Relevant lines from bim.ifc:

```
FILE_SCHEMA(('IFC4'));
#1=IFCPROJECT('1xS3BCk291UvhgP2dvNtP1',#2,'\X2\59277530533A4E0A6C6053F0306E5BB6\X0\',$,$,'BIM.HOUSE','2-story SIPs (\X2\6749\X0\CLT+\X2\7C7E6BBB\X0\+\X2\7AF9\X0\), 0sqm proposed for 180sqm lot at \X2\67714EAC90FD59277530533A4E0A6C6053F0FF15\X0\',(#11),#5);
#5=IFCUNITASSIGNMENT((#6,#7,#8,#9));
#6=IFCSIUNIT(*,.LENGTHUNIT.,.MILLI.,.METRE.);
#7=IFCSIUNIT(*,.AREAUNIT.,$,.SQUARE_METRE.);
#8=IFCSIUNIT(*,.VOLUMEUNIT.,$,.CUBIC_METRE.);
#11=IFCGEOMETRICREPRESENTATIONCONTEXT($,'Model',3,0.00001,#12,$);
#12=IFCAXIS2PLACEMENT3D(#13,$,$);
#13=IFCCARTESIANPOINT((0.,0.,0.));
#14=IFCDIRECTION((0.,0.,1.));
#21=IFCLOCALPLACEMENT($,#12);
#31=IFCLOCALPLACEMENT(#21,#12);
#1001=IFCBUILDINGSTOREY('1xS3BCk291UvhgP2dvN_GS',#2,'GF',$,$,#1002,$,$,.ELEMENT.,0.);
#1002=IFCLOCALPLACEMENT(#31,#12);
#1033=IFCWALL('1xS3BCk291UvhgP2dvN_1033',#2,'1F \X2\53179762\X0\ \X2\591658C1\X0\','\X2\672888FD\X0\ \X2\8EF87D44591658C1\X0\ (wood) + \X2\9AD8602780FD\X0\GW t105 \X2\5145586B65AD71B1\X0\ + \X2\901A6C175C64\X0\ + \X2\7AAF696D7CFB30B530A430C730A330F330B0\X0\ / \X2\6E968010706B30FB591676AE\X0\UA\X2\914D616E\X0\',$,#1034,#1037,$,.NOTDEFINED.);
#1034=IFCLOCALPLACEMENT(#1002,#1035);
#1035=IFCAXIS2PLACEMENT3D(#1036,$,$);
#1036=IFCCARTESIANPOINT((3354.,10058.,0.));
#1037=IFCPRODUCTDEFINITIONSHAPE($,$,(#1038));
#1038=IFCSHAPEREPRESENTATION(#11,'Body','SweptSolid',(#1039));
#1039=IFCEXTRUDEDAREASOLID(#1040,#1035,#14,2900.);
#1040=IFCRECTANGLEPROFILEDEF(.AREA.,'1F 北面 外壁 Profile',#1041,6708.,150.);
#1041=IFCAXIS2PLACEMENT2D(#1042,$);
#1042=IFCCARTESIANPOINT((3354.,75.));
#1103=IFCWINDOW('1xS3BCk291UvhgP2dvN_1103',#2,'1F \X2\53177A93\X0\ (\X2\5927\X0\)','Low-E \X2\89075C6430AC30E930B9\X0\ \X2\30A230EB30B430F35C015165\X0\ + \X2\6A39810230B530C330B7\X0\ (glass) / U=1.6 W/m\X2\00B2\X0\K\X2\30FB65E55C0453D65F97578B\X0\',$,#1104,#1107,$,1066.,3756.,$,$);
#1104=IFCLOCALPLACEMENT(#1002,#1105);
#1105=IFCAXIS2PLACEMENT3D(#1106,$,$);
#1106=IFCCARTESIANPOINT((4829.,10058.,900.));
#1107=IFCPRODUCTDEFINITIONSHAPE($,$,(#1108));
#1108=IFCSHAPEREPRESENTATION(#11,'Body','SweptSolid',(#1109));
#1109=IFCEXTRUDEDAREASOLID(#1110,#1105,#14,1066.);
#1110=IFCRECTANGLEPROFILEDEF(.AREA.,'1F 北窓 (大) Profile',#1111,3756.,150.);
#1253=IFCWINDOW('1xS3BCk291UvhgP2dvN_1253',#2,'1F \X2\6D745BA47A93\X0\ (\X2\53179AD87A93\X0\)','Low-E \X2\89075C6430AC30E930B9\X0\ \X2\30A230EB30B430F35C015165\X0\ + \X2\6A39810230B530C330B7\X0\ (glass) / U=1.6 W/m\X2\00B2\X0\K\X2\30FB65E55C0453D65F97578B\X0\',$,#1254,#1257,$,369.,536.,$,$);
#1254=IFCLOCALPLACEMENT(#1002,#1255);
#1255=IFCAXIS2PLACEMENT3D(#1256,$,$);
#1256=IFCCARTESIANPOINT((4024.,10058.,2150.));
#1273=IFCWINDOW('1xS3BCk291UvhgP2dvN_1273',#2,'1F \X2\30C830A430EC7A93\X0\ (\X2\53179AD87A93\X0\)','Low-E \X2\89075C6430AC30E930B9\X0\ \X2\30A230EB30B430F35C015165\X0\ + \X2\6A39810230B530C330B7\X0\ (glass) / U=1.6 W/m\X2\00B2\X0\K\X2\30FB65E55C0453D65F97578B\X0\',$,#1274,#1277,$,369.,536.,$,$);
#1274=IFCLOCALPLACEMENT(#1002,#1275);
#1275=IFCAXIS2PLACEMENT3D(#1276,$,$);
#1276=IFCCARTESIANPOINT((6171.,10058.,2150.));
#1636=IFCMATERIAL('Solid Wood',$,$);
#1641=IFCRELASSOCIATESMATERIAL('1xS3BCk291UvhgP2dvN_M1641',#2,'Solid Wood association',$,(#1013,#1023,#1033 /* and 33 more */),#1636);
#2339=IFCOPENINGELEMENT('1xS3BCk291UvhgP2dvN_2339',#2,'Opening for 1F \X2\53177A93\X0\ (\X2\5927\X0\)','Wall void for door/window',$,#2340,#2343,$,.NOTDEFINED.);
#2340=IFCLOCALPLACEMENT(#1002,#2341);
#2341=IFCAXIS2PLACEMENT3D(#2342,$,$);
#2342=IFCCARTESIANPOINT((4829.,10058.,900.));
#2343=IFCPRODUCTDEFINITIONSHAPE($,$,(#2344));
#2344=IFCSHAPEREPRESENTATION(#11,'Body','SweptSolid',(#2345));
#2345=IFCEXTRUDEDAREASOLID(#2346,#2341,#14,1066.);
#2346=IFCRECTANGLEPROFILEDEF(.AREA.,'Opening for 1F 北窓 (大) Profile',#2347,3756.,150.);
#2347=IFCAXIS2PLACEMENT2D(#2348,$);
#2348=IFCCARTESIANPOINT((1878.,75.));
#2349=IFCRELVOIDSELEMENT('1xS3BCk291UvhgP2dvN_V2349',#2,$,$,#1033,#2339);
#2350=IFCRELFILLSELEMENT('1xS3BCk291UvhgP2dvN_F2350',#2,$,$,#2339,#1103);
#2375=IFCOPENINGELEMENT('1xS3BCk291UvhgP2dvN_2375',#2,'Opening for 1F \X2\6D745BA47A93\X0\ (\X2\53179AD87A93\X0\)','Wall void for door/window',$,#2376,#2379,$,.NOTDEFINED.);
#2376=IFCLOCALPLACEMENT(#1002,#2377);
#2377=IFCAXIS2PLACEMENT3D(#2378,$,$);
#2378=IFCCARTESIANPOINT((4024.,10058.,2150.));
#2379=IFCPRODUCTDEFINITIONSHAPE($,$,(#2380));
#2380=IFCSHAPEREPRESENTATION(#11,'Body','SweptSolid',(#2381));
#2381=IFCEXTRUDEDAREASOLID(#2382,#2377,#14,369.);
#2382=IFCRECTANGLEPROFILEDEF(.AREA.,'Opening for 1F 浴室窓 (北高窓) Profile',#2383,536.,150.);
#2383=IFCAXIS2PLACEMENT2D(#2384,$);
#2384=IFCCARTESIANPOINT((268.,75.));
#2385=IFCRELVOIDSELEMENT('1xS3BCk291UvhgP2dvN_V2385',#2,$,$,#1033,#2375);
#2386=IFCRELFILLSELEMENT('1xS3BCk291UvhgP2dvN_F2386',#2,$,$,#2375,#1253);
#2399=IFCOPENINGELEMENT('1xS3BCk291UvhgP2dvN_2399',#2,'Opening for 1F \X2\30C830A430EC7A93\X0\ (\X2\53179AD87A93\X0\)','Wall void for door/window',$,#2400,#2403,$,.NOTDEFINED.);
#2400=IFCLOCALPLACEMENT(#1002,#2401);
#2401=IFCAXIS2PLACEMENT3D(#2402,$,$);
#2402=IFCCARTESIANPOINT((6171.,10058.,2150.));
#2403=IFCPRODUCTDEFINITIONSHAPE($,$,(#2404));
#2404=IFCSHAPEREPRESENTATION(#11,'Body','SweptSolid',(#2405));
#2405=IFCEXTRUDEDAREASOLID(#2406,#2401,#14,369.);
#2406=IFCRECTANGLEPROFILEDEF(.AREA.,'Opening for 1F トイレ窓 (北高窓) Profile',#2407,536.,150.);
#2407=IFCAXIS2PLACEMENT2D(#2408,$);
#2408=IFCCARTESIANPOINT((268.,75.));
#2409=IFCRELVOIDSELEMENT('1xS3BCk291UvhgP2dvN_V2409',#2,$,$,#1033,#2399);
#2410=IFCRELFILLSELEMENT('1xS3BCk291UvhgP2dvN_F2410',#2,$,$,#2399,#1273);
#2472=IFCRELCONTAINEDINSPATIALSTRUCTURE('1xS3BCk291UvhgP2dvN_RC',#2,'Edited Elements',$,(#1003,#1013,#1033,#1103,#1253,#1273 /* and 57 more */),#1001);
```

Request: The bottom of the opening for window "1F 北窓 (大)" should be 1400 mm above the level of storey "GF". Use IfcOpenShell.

```python
import numpy as np
import ifcopenshell
import ifcopenshell.api.geometry
import ifcopenshell.geom
import ifcopenshell.util.element
import ifcopenshell.util.placement
import ifcopenshell.util.shape
import ifcopenshell.util.unit

model = ifcopenshell.open("bim.ifc")
unit_scale = ifcopenshell.util.unit.calculate_unit_scale(model)

window = model.by_guid("1xS3BCk291UvhgP2dvN_1103")
opening = window.FillsVoids[0].RelatingOpeningElement
storey = ifcopenshell.util.element.get_container(window, ifc_class="IfcBuildingStorey")
level = ifcopenshell.util.placement.get_local_placement(storey.ObjectPlacement)[2, 3]

# The opening's origin need not be at the sill, so measure its lowest point.
shape = ifcopenshell.geom.create_shape(ifcopenshell.geom.settings(), opening)
bottom = ifcopenshell.util.shape.get_shape_bottom_elevation(shape, shape.geometry) / unit_scale
dz = level + 1.4 / unit_scale - bottom

shift = np.array([0.0, 0.0, dz])
# The window is not placed relative to its opening, so move both.
for product in (opening, window):
    matrix = ifcopenshell.util.placement.get_local_placement(product.ObjectPlacement)
    matrix[:3, 3] += shift
    ifcopenshell.api.geometry.edit_object_placement(model, product=product, matrix=matrix, is_si=False)

print(f"moved by {dz * unit_scale:+.3f} m")

model.write("bim_edited.ifc")
```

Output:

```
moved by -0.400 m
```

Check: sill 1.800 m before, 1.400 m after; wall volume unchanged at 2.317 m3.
